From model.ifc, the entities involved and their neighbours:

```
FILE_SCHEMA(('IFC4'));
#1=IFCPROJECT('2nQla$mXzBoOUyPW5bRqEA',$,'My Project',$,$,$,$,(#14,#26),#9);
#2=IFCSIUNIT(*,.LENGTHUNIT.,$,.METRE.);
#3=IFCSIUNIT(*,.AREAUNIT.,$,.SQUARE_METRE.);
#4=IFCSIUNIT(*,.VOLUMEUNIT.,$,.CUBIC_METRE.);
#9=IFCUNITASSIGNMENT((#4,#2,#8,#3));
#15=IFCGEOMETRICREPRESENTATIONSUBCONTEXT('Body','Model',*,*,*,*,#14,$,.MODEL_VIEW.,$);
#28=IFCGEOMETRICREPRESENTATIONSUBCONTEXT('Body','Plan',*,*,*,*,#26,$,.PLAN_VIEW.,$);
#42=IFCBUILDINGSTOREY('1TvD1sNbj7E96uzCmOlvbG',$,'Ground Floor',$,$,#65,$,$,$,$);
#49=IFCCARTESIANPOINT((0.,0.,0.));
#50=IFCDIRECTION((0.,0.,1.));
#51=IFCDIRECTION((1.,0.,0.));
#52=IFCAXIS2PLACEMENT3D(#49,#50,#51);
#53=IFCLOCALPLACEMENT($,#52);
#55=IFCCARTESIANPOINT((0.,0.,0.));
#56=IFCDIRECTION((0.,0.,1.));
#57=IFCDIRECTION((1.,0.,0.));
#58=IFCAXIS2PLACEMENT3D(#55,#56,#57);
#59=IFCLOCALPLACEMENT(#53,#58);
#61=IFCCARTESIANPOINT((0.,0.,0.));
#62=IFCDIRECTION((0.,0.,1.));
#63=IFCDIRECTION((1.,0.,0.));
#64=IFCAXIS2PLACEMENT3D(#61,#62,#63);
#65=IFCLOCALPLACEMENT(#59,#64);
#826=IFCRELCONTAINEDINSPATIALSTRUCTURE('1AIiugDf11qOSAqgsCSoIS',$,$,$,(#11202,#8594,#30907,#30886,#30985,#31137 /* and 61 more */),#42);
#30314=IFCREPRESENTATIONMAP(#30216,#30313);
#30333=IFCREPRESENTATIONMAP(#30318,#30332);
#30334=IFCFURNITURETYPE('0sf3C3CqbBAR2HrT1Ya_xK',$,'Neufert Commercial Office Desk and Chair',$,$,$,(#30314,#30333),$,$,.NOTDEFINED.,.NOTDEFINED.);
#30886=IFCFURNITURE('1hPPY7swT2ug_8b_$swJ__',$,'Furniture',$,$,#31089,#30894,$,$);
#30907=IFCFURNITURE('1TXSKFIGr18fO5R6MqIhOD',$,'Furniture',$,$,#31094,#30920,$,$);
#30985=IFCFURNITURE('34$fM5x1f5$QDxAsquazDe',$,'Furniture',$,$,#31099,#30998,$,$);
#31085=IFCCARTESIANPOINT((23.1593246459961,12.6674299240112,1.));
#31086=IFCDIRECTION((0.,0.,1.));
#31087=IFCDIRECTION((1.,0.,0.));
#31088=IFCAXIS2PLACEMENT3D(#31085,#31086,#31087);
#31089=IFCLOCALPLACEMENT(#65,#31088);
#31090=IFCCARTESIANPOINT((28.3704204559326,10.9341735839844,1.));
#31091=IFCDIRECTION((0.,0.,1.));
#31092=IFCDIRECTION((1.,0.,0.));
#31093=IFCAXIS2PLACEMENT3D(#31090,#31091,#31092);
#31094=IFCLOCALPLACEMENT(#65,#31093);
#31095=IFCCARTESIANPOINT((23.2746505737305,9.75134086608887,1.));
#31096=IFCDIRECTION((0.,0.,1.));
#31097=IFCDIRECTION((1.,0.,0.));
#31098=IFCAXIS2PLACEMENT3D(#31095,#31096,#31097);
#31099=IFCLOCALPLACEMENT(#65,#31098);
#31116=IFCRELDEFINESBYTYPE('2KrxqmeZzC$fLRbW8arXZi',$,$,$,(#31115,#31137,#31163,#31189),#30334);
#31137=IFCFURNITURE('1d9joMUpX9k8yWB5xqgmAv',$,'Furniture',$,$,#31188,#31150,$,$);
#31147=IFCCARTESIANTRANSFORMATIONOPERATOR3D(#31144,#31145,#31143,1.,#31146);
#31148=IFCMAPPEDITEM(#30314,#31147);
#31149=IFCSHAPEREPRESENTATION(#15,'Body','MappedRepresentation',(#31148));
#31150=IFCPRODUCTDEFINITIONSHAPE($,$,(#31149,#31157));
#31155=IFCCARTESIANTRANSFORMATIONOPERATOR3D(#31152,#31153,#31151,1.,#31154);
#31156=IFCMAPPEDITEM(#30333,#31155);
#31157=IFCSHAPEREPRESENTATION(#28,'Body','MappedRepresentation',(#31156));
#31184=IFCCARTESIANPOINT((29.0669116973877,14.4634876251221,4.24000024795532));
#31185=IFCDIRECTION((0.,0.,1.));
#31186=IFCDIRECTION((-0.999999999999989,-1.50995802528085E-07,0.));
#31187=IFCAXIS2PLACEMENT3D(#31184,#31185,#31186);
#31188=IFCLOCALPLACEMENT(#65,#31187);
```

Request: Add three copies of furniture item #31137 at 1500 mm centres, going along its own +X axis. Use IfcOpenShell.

```python
import ifcopenshell
import ifcopenshell.api.geometry
import ifcopenshell.api.root
import ifcopenshell.util.element
import ifcopenshell.util.placement
import ifcopenshell.util.unit

model = ifcopenshell.open("model.ifc")
unit_scale = ifcopenshell.util.unit.calculate_unit_scale(model)

source = model.by_guid("1d9joMUpX9k8yWB5xqgmAv")
base = ifcopenshell.util.placement.get_local_placement(source.ObjectPlacement)
step = base[:3, 0] * 1.5 / unit_scale

for i in range(1, 4):
    copy = ifcopenshell.api.root.copy_class(model, product=source)
    copy.Representation = ifcopenshell.util.element.copy_deep(
        model, source.Representation, exclude=["IfcGeometricRepresentationContext", "IfcRepresentationMap"]
    )
    matrix = base.copy()
    matrix[:3, 3] += i * step
    print("added at", matrix[:3, 3].round(3) + 0.0)
    ifcopenshell.api.geometry.edit_object_placement(model, product=copy, matrix=matrix, is_si=False)

model.write("model-out.ifc")
```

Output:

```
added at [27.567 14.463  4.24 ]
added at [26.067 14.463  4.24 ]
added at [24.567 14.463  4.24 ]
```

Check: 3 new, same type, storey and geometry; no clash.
